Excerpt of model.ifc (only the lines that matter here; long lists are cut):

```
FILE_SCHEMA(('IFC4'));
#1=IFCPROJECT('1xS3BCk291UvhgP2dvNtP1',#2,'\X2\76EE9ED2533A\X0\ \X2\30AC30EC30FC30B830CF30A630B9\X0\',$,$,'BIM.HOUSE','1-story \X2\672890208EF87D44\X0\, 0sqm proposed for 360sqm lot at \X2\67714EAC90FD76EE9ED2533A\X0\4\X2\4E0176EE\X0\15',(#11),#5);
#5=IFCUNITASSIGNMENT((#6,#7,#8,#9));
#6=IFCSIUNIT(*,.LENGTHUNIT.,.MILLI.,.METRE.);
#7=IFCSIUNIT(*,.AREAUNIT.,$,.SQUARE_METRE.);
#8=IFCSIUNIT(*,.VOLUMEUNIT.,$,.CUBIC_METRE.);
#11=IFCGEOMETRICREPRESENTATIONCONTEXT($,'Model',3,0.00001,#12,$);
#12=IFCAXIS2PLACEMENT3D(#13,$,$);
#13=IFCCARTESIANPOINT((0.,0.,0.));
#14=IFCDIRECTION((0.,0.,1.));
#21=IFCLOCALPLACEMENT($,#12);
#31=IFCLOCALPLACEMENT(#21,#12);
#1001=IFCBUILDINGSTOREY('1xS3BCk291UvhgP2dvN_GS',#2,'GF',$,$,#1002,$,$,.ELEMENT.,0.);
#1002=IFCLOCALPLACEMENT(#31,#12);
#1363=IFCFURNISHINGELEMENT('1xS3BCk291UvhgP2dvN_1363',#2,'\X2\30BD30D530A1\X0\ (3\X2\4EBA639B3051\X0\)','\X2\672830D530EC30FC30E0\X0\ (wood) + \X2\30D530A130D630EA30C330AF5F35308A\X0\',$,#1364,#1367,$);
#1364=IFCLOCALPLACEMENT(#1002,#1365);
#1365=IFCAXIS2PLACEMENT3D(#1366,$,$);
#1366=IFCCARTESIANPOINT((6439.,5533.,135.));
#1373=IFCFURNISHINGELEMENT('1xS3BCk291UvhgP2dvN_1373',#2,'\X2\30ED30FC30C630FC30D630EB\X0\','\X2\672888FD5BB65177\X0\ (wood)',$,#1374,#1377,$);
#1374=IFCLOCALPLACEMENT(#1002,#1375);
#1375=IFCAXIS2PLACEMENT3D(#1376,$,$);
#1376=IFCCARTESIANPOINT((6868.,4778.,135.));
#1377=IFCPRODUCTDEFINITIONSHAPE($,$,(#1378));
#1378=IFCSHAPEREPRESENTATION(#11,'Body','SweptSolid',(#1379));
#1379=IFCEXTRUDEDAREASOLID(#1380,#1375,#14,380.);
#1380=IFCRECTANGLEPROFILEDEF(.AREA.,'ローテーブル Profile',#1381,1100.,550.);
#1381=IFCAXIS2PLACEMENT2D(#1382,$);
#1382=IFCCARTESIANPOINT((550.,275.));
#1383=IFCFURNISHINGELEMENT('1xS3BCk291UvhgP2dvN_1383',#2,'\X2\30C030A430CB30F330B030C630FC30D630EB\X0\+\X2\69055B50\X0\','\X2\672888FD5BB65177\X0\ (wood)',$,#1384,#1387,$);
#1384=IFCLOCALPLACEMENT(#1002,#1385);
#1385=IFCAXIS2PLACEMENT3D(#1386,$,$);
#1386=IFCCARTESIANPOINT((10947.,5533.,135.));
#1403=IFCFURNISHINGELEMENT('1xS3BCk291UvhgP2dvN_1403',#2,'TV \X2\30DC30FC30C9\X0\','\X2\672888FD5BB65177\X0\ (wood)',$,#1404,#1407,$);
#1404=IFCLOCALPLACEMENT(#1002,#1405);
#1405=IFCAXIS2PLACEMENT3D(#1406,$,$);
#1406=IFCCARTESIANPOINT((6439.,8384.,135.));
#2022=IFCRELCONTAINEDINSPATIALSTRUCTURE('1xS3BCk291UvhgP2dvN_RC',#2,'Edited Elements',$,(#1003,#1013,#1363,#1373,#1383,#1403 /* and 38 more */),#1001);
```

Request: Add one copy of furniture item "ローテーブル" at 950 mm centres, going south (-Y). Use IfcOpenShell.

```python
import numpy as np
import ifcopenshell
import ifcopenshell.api.geometry
import ifcopenshell.api.root
import ifcopenshell.util.element
import ifcopenshell.util.placement
import ifcopenshell.util.unit

model = ifcopenshell.open("model.ifc")
unit_scale = ifcopenshell.util.unit.calculate_unit_scale(model)


def reuse_history(source, copy):
    """copy_class also copies each property set's owner history, people and application; keep the originals."""
    for rel in copy.IsDefinedBy:
        if rel.is_a("IfcRelDefinesByProperties") and (history := rel.RelatingPropertyDefinition.OwnerHistory):
            rel.RelatingPropertyDefinition.OwnerHistory = source.OwnerHistory
            ifcopenshell.util.element.remove_deep2(model, history)


source = model.by_guid("1xS3BCk291UvhgP2dvN_1373")
base = ifcopenshell.util.placement.get_local_placement(source.ObjectPlacement)
step = np.array([0.0, -1.0, 0.0]) * 0.95 / unit_scale

for i in range(1, 2):
    copy = ifcopenshell.api.root.copy_class(model, product=source)
    copy.Representation = ifcopenshell.util.element.copy_deep(
        model, source.Representation, exclude=["IfcGeometricRepresentationContext", "IfcRepresentationMap"]
    )
    reuse_history(source, copy)
    matrix = base.copy()
    matrix[:3, 3] += i * step
    print("added at", matrix[:3, 3].round(3) + 0.0)
    ifcopenshell.api.geometry.edit_object_placement(model, product=copy, matrix=matrix, is_si=False)

model.write("model_v2.ifc")
```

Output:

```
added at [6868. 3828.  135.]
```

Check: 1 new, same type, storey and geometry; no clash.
